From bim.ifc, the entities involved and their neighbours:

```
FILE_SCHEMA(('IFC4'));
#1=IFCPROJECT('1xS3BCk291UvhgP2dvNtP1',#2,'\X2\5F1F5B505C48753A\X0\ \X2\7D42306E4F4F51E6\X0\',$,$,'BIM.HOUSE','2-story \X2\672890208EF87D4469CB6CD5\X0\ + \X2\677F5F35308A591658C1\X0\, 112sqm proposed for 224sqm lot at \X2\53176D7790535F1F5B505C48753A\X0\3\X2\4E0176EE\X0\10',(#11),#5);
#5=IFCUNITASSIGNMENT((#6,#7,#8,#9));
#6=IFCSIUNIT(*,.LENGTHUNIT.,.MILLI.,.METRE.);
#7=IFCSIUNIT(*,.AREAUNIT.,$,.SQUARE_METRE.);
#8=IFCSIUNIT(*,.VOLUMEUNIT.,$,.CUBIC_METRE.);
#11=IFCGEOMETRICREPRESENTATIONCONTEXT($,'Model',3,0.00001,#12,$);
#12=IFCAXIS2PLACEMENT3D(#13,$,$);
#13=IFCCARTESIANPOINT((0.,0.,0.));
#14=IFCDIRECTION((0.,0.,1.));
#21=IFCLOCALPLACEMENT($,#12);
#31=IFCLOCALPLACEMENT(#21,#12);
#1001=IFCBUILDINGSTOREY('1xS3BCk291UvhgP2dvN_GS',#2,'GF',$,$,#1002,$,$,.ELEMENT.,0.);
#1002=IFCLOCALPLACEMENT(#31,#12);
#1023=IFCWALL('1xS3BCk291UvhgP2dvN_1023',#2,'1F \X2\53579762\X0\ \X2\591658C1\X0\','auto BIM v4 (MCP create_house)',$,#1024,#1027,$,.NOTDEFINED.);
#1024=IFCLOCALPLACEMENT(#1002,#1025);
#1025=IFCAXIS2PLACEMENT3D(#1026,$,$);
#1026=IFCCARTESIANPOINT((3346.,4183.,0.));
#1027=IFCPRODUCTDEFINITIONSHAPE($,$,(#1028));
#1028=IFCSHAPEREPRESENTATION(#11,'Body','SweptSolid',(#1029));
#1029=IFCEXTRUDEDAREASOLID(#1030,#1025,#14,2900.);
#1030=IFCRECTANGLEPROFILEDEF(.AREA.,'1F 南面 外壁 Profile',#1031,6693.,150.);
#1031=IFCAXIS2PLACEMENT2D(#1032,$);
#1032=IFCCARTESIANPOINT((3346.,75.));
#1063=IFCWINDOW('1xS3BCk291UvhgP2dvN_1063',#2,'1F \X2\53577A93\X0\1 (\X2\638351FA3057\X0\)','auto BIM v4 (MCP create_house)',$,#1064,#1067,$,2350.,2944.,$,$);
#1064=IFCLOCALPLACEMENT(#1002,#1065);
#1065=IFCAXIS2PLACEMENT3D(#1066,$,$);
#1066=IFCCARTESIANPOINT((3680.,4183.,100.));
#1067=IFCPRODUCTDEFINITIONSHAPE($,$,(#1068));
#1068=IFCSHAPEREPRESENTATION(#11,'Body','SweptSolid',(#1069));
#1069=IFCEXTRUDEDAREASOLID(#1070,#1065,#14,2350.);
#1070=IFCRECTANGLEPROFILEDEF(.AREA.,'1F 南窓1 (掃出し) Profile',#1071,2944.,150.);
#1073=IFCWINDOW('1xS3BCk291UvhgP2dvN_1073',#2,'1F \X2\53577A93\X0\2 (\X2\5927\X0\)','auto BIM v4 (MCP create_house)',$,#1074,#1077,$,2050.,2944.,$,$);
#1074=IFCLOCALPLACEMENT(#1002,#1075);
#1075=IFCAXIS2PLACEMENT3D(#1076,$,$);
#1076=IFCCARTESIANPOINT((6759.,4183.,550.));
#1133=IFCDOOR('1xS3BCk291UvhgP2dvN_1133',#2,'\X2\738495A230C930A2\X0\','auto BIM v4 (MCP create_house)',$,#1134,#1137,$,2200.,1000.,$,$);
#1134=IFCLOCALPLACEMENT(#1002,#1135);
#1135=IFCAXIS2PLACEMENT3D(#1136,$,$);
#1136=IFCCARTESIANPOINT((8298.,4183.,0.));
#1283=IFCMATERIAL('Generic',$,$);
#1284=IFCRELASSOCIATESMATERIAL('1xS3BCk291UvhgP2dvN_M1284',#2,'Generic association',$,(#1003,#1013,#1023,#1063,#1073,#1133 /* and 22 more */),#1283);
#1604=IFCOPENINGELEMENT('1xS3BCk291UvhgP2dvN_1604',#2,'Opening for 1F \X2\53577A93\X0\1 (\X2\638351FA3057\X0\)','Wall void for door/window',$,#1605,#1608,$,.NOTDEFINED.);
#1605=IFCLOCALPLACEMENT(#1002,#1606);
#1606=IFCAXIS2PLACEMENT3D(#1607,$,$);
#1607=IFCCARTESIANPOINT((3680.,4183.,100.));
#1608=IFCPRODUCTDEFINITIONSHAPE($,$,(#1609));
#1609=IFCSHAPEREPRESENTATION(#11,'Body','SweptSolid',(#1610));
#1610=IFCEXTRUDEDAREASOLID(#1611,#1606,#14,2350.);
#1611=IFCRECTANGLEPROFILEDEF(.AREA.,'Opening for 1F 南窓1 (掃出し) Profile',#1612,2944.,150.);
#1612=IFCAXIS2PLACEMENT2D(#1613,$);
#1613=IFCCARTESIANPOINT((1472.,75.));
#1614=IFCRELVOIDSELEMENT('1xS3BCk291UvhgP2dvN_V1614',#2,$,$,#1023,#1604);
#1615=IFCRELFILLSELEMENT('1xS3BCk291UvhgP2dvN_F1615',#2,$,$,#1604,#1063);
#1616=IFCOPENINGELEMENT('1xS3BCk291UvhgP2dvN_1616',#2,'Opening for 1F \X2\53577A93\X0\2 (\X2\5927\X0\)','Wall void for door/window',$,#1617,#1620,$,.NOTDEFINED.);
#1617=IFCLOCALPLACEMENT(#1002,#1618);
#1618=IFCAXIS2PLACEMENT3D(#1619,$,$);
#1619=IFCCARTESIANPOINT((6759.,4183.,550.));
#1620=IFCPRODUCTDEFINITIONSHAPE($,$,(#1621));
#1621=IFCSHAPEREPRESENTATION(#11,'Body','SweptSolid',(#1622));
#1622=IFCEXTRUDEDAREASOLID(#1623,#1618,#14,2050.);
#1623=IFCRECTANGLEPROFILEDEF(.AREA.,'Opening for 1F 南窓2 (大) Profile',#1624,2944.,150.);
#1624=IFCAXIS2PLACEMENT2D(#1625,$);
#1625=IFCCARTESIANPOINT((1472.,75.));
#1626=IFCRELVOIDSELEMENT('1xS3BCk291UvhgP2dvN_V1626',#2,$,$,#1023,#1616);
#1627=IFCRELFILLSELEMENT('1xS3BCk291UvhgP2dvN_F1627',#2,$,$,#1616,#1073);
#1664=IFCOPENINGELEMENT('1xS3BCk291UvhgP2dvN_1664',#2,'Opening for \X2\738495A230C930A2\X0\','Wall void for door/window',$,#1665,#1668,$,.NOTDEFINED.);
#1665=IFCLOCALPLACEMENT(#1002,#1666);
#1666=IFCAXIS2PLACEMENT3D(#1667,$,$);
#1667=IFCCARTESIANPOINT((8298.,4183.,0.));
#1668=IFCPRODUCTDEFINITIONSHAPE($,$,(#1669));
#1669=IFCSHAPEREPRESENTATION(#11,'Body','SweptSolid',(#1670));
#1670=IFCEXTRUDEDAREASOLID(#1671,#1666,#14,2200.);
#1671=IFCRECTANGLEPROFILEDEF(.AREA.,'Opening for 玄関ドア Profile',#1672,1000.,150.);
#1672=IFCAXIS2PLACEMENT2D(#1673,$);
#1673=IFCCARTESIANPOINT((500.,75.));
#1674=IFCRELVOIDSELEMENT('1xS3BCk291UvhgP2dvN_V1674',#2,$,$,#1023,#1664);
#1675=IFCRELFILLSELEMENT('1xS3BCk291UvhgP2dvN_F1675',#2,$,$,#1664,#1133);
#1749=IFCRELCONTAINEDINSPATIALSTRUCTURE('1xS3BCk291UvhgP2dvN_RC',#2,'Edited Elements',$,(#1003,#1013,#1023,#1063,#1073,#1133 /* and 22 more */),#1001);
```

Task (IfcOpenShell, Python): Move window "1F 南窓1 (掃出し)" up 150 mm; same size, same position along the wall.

```python
import numpy as np
import ifcopenshell
import ifcopenshell.api.geometry
import ifcopenshell.util.placement
import ifcopenshell.util.unit

model = ifcopenshell.open("bim.ifc")
unit_scale = ifcopenshell.util.unit.calculate_unit_scale(model)

window = model.by_guid("1xS3BCk291UvhgP2dvN_1063")
opening = window.FillsVoids[0].RelatingOpeningElement
dz = 150.0

shift = np.array([0.0, 0.0, dz])
# The window is not placed relative to its opening, so move both.
for product in (opening, window):
    matrix = ifcopenshell.util.placement.get_local_placement(product.ObjectPlacement)
    matrix[:3, 3] += shift
    ifcopenshell.api.geometry.edit_object_placement(model, product=product, matrix=matrix, is_si=False)

print(f"moved by {dz * unit_scale:+.3f} m")

model.write("bim_edited.ifc")
```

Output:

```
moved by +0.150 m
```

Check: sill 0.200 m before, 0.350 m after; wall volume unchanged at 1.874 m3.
